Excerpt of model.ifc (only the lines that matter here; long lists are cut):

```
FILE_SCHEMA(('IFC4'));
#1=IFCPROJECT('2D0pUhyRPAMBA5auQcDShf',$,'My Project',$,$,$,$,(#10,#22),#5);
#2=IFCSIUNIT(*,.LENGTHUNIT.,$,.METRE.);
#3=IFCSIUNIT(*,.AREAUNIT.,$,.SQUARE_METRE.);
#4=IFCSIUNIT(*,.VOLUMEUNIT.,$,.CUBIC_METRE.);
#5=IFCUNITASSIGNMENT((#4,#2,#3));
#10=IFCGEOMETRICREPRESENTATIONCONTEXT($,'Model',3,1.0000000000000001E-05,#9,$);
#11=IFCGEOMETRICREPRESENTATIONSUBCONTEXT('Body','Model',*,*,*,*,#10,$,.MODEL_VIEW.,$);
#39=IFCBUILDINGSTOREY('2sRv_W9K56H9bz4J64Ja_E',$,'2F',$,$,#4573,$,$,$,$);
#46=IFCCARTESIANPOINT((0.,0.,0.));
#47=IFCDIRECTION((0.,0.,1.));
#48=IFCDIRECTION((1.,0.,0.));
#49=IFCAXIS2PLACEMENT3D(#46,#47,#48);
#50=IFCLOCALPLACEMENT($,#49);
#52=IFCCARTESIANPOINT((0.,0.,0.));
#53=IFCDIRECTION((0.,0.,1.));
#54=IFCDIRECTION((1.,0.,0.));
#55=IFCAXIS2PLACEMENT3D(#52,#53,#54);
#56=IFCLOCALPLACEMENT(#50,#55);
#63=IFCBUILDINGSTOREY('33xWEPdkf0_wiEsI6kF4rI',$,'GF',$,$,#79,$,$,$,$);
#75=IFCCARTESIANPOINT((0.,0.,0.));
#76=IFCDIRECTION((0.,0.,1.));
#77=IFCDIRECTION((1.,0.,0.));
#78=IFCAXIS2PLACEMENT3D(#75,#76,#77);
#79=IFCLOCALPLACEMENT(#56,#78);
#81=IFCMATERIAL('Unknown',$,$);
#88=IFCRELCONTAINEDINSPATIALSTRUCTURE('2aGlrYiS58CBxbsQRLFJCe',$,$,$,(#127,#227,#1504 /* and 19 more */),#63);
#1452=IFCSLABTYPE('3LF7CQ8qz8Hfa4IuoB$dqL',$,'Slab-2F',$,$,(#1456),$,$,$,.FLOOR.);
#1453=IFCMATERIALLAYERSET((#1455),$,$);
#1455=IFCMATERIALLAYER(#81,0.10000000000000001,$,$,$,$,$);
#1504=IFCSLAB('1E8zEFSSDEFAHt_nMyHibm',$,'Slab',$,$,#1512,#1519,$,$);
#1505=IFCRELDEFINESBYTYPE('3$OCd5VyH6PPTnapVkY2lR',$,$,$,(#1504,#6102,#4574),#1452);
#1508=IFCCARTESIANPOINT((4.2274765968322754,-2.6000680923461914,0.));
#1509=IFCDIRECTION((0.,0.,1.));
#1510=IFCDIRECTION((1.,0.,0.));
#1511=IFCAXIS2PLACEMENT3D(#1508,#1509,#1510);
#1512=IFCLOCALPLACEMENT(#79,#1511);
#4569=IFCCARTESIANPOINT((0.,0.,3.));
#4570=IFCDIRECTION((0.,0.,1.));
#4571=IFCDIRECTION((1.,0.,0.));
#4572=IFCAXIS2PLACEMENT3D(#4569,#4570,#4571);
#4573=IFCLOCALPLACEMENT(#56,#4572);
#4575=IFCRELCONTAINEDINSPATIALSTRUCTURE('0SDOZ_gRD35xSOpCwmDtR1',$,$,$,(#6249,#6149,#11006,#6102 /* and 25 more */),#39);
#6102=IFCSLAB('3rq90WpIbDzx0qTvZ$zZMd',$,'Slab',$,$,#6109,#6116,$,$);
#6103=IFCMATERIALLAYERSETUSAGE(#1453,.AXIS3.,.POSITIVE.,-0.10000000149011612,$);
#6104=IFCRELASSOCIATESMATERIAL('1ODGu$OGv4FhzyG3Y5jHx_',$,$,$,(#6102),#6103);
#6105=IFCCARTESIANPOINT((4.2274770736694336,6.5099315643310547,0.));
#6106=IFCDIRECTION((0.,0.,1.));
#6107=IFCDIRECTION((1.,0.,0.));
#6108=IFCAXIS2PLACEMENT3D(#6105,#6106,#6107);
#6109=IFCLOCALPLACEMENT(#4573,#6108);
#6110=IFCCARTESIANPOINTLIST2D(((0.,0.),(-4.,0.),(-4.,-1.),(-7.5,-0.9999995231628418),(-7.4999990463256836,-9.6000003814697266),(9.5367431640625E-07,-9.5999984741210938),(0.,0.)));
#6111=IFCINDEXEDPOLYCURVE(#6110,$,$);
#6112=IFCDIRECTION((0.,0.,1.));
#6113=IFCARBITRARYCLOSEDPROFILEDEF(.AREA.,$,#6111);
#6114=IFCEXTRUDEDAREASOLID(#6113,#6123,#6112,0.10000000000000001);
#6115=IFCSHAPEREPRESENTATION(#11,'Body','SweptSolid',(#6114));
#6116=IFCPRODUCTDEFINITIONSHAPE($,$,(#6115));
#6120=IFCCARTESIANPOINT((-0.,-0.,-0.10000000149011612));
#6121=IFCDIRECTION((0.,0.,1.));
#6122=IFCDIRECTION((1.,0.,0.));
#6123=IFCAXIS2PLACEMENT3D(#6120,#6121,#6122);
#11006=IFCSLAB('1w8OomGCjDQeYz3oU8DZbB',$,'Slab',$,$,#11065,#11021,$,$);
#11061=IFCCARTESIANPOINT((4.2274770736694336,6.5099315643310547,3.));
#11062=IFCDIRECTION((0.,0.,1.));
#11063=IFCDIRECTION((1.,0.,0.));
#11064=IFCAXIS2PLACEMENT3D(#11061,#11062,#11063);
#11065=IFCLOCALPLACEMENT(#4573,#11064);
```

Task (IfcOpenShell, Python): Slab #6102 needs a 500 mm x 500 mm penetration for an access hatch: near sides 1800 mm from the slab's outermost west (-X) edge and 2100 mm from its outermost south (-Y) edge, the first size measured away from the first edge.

```python
import numpy as np
import ifcopenshell
import ifcopenshell.api.feature
import ifcopenshell.api.geometry
import ifcopenshell.api.root
import ifcopenshell.geom
import ifcopenshell.util.placement
import ifcopenshell.util.representation
import ifcopenshell.util.shape
import ifcopenshell.util.unit

model = ifcopenshell.open("model.ifc")
unit_scale = ifcopenshell.util.unit.calculate_unit_scale(model)
settings = ifcopenshell.geom.settings()


def volume(element):
    """Net volume in cubic metres, openings subtracted."""
    shape = ifcopenshell.geom.create_shape(settings, element)
    return ifcopenshell.util.shape.get_volume(shape.geometry)


slab = model.by_guid("3rq90WpIbDzx0qTvZ$zZMd")
before = volume(slab)

# Extent in the slab's own axes, in metres. The edges named are its -X and -Y sides.
slab_shape = ifcopenshell.geom.create_shape(settings, slab)
vertices = ifcopenshell.util.shape.get_vertices(slab_shape.geometry)
x_min, y_min, bottom = vertices.min(axis=0)
top = vertices[:, 2].max()

opening = ifcopenshell.api.root.create_entity(model, ifc_class="IfcOpeningElement", name="Access hatch opening", predefined_type="OPENING")
context = ifcopenshell.util.representation.get_context(model, "Model", "Body", "MODEL_VIEW")
width, depth = 0.5, 0.5
outline = [(0.0, 0.0), (width, 0.0), (width, depth), (0.0, depth), (0.0, 0.0)]
# Overshoot both faces by 50 mm so the cut is clean.
shape = ifcopenshell.api.geometry.add_slab_representation(
    model, context=context, depth=top - bottom + 0.1, polyline=outline
)
ifcopenshell.api.geometry.assign_representation(model, product=opening, representation=shape)

matrix = ifcopenshell.util.placement.get_local_placement(slab.ObjectPlacement)
matrix[:, 3] = matrix @ np.append(np.array([x_min + 1.8, y_min + 2.1, bottom - 0.05]) / unit_scale, 1.0)
ifcopenshell.api.geometry.edit_object_placement(model, product=opening, matrix=matrix, is_si=False)
ifcopenshell.api.feature.add_feature(model, feature=opening, element=slab)

after = volume(slab)

print(f"slab volume {before:.3f} -> {after:.3f} m3")

model.write("model_updated.ifc")
```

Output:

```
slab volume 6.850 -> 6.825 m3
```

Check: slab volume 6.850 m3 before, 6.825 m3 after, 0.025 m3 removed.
